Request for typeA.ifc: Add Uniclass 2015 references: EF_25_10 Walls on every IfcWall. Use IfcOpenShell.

First a look at what the model holds.

```python
import ifcopenshell

model = ifcopenshell.open("typeA.ifc")
print(model.schema)
print("classifications:", [c.Name for c in model.by_type("IfcClassification")])
for ifc_class in ("IfcDoor", "IfcRoof", "IfcStair", "IfcWall", "IfcWindow"):
    print(ifc_class, len(model.by_type(ifc_class)))
```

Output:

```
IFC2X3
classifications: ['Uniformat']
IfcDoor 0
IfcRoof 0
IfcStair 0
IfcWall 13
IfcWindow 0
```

```python
import ifcopenshell
import ifcopenshell.api.classification

model = ifcopenshell.open("typeA.ifc")

# IFC2X3 requires Source and Edition and has no link from the project to the system.
system = model.create_entity("IfcClassification", Source="NBS", Edition="2015", Name="Uniclass 2015")

codes = {
    "IfcWall": ("EF_25_10", "Walls"),
}
for ifc_class, (code, name) in codes.items():
    products = model.by_type(ifc_class)
    ifcopenshell.api.classification.add_reference(
        model, products=products, classification=system, identification=code, name=name
    )
    print(code, len(products))

model.write("typeA_rev.ifc")
```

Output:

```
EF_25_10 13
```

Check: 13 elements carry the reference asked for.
